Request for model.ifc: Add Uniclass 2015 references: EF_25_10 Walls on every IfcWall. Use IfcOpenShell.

First a look at what the model holds.

```python
import ifcopenshell

model = ifcopenshell.open("model.ifc")
print(model.schema)
print("classifications:", [c.Name for c in model.by_type("IfcClassification")])
for ifc_class in ("IfcDoor", "IfcRoof", "IfcStair", "IfcWall", "IfcWindow"):
    print(ifc_class, len(model.by_type(ifc_class)))
```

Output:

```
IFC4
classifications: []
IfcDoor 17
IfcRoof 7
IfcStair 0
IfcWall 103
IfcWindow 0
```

```python
import ifcopenshell
import ifcopenshell.api.classification

model = ifcopenshell.open("model.ifc")

system = ifcopenshell.api.classification.add_classification(model, classification="Uniclass 2015")

codes = {
    "IfcWall": ("EF_25_10", "Walls"),
}
for ifc_class, (code, name) in codes.items():
    products = model.by_type(ifc_class)
    ifcopenshell.api.classification.add_reference(
        model, products=products, classification=system, identification=code, name=name
    )
    print(code, len(products))

model.write("model_edited.ifc")
```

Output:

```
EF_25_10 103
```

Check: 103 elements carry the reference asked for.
